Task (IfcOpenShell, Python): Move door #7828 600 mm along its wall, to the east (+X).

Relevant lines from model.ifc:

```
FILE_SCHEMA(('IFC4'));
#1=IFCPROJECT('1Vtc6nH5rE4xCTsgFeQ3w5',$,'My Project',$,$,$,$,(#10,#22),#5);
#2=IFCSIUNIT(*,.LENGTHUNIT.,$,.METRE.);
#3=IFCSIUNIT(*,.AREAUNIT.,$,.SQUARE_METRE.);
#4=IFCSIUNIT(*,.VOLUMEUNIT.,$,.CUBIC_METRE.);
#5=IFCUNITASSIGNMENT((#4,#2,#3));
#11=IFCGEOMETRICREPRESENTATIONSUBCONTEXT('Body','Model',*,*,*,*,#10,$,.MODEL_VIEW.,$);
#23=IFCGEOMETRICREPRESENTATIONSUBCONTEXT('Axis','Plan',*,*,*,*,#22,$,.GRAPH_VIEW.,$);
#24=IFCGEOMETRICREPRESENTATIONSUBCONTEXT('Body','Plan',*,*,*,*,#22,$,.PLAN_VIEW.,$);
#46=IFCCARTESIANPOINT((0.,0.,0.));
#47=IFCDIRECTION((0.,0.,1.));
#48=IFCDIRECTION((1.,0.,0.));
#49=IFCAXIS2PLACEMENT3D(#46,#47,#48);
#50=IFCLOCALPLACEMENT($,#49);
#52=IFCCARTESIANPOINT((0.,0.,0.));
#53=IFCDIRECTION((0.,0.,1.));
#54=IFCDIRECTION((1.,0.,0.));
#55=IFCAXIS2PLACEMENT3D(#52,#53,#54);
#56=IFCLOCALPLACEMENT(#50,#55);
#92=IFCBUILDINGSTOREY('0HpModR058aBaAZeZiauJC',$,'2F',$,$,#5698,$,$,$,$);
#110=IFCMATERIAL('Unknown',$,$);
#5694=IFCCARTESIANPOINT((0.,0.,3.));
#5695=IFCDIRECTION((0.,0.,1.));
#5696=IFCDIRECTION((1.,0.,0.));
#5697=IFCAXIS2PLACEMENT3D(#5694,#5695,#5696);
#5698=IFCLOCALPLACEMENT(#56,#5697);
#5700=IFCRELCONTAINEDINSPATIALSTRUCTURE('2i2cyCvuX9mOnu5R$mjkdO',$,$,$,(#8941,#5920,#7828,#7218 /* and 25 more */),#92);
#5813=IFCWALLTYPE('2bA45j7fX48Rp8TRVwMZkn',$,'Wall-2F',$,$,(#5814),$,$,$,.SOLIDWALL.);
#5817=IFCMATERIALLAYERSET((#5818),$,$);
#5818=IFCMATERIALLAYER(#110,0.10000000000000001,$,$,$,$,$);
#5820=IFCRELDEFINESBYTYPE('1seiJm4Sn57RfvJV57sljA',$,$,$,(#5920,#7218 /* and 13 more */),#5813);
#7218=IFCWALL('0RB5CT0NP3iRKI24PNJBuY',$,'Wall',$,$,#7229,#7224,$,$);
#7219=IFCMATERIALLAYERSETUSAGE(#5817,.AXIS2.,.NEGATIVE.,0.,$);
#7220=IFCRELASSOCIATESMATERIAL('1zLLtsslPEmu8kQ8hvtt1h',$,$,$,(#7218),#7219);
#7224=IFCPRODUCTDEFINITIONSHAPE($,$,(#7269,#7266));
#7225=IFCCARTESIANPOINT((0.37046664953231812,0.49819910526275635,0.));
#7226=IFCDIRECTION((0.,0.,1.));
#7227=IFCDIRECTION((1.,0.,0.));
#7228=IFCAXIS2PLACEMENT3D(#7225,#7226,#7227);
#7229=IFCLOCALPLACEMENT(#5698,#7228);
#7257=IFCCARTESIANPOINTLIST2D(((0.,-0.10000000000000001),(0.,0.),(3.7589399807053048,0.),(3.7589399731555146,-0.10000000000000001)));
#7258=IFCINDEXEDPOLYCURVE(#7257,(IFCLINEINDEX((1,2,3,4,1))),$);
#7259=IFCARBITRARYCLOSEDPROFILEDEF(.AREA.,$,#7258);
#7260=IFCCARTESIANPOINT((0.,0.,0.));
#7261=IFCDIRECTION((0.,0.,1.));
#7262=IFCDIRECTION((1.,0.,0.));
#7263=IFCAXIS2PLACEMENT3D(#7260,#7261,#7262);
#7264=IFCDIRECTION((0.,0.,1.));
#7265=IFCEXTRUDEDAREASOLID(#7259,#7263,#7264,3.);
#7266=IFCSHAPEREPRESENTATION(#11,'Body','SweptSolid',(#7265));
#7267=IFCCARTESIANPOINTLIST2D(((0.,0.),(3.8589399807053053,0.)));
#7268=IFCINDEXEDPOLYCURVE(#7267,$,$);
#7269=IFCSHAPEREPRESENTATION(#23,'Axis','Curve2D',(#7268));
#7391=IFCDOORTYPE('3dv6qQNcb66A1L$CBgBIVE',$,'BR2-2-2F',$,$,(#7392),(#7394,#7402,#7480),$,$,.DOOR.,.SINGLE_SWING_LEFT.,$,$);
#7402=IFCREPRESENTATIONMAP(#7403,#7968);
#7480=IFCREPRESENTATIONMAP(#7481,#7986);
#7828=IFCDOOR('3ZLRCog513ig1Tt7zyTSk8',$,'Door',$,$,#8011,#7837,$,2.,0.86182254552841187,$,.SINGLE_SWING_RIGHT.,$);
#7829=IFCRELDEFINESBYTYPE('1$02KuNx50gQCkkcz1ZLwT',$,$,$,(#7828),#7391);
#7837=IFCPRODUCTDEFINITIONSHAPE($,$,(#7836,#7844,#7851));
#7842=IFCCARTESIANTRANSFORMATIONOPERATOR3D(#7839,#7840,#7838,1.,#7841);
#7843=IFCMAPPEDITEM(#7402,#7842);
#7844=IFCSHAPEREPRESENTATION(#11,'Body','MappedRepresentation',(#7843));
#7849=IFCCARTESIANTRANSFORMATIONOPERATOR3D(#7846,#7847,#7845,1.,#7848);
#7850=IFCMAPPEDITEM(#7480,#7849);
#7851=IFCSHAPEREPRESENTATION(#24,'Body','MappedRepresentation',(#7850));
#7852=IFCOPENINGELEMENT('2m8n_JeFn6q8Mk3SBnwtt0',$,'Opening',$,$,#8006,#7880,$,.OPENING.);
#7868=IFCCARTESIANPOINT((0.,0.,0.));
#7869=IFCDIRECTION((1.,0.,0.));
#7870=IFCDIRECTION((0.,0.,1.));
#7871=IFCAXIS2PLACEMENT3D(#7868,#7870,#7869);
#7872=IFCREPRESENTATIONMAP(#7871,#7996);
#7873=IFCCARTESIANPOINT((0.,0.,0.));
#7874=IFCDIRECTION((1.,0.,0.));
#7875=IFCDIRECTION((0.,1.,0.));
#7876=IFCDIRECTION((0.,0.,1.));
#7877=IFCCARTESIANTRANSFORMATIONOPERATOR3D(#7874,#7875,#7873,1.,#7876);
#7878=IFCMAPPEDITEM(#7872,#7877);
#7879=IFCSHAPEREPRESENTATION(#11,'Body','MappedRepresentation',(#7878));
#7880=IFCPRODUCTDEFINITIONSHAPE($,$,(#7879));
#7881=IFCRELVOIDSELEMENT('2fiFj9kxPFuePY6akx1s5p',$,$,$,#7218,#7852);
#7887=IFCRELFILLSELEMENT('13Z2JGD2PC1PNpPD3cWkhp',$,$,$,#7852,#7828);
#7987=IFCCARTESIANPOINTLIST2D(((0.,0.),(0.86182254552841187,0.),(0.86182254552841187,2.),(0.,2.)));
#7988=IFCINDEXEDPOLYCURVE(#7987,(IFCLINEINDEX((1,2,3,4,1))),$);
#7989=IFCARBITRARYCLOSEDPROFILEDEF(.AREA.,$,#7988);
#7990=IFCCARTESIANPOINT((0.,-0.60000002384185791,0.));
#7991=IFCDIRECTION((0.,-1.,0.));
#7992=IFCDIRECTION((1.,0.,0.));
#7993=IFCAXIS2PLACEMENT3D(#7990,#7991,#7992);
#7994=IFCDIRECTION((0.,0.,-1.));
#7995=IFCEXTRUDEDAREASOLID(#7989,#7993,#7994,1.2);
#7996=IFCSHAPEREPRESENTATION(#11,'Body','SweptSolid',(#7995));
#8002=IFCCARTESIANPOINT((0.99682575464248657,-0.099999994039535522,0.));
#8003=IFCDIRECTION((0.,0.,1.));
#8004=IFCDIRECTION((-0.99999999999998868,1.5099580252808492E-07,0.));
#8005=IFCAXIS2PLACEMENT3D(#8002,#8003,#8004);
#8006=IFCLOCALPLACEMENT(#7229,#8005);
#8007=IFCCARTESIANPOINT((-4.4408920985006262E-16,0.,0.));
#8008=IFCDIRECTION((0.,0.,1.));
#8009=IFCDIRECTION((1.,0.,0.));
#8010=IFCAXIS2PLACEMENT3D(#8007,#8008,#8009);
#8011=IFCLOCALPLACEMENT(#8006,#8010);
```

```python
import ifcopenshell
import ifcopenshell.api.geometry
import ifcopenshell.util.placement
import ifcopenshell.util.unit

model = ifcopenshell.open("model.ifc")
unit_scale = ifcopenshell.util.unit.calculate_unit_scale(model)

door = model.by_guid("3ZLRCog513ig1Tt7zyTSk8")
opening = door.FillsVoids[0].RelatingOpeningElement
wall = opening.VoidsElements[0].RelatingBuildingElement

wall_matrix = ifcopenshell.util.placement.get_local_placement(wall.ObjectPlacement)
shift = wall_matrix[:3, 0] * 0.6 / unit_scale
before = ifcopenshell.util.placement.get_local_placement(door.ObjectPlacement)[:3, 3].copy()

# The door is placed relative to its opening, so it follows when the opening moves.
matrix = ifcopenshell.util.placement.get_local_placement(opening.ObjectPlacement)
matrix[:3, 3] += shift
ifcopenshell.api.geometry.edit_object_placement(
    model, product=opening, matrix=matrix, is_si=False, should_transform_children=True
)

after = ifcopenshell.util.placement.get_local_placement(door.ObjectPlacement)[:3, 3]
print("door moved by", (after - before).round(3) + 0.0)

model.write("model_rev.ifc")
```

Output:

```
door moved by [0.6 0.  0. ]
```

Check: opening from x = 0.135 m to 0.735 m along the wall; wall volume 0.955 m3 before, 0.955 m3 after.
